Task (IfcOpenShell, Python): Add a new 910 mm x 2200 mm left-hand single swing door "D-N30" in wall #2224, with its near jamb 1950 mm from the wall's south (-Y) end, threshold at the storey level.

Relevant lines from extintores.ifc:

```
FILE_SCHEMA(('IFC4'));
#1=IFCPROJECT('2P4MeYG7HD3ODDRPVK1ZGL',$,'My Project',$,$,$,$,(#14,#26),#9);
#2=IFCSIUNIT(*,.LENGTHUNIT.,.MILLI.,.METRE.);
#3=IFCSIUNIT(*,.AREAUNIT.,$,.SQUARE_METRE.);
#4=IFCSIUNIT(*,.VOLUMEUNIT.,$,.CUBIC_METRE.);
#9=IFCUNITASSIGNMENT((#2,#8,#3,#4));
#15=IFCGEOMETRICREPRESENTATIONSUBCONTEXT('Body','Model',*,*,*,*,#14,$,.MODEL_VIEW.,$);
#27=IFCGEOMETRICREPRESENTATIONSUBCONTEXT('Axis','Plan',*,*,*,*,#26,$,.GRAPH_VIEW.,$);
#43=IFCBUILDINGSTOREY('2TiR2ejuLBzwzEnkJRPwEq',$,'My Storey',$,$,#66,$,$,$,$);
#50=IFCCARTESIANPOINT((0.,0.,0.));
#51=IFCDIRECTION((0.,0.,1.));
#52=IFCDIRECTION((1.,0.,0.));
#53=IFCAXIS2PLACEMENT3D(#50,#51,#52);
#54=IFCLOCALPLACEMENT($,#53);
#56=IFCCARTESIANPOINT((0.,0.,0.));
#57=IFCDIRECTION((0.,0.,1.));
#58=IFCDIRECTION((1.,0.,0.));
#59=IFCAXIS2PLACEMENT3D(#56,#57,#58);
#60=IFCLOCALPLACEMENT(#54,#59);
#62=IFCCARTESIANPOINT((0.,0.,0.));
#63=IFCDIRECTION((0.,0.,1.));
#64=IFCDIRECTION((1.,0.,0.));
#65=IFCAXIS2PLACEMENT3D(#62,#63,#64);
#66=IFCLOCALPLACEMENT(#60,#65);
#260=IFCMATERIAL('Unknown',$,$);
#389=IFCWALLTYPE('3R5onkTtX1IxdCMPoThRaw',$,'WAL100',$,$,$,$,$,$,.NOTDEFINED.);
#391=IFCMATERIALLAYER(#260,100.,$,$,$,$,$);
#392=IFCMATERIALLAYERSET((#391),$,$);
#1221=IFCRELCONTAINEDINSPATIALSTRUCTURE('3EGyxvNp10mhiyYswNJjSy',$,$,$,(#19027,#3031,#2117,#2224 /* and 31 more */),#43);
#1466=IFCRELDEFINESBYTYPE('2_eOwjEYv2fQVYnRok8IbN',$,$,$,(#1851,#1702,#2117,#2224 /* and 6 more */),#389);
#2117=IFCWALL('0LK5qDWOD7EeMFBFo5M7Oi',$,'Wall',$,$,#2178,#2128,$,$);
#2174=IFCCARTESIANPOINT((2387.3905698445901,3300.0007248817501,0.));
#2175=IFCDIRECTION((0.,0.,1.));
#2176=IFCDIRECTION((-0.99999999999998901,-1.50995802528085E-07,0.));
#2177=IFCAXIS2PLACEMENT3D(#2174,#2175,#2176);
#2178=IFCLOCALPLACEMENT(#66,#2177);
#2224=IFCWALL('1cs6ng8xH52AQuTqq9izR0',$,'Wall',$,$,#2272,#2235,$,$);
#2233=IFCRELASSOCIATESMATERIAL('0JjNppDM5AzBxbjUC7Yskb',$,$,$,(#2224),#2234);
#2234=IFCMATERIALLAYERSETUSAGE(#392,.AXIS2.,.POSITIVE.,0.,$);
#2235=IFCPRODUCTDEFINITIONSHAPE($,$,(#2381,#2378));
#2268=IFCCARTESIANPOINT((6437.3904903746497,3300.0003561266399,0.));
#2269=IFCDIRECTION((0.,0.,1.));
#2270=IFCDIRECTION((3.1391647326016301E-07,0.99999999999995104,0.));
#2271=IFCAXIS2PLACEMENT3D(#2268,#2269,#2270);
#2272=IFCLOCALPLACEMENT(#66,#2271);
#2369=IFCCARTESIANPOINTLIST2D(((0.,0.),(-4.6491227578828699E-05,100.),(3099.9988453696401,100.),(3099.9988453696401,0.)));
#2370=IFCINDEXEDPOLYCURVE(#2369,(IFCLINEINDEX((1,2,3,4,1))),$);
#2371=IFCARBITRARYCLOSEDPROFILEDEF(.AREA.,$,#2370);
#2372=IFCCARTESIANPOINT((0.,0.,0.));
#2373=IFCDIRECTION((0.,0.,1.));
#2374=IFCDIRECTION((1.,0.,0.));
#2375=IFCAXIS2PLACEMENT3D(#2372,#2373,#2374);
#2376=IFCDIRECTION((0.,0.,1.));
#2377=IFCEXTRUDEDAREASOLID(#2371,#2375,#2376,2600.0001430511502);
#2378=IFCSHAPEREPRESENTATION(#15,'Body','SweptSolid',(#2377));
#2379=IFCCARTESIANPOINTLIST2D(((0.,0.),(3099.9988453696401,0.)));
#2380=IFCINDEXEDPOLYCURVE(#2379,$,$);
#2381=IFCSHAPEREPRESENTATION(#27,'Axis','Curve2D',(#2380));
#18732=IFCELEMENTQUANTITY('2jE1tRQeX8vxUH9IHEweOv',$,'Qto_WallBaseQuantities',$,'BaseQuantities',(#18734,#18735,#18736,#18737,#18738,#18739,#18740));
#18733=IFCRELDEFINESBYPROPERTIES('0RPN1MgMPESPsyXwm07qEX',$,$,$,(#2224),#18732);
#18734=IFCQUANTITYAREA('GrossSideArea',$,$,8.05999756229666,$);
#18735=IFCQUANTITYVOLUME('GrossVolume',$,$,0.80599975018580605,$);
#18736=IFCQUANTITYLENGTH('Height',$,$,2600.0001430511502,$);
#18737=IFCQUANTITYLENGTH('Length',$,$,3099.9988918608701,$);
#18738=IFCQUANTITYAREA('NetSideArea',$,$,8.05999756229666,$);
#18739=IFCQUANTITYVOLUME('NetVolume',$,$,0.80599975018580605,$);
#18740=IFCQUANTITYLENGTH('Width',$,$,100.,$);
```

```python
import numpy as np
import ifcopenshell
import ifcopenshell.api.feature
import ifcopenshell.api.geometry
import ifcopenshell.api.pset
import ifcopenshell.api.root
import ifcopenshell.api.spatial
import ifcopenshell.geom
import ifcopenshell.util.element
import ifcopenshell.util.placement
import ifcopenshell.util.representation
import ifcopenshell.util.shape
import ifcopenshell.util.unit

model = ifcopenshell.open("extintores.ifc")
unit_scale = ifcopenshell.util.unit.calculate_unit_scale(model)
area_scale = ifcopenshell.util.unit.calculate_unit_scale(model, "AREAUNIT")
volume_scale = ifcopenshell.util.unit.calculate_unit_scale(model, "VOLUMEUNIT")
settings = ifcopenshell.geom.settings()


def volume(element):
    """Net volume in cubic metres, openings subtracted."""
    shape = ifcopenshell.geom.create_shape(settings, element)
    return ifcopenshell.util.shape.get_volume(shape.geometry)


wall = model.by_guid("1cs6ng8xH52AQuTqq9izR0")
storey = ifcopenshell.util.element.get_container(wall, ifc_class="IfcBuildingStorey")
context = ifcopenshell.util.representation.get_context(model, "Model", "Body", "MODEL_VIEW")
before = volume(wall)

width, height, from_end, sill = 0.91, 2.2, 1.95, 0.0  # metres

# The wall runs along its own X axis, and the end named is its -X end.
wall_shape = ifcopenshell.geom.create_shape(settings, wall)
x, y, z = ifcopenshell.util.shape.get_vertices(wall_shape.geometry).T
start = x.min() + from_end
face, thickness = float(y.min()), float(y.max() - y.min())
wall_matrix = ifcopenshell.util.placement.get_local_placement(wall.ObjectPlacement)
level = ifcopenshell.util.placement.get_local_placement(storey.ObjectPlacement)[2, 3]


def in_wall(x, y):
    """Placement at x, y metres in the wall's axes, at sill height."""
    matrix = wall_matrix.copy()
    matrix[:, 3] = wall_matrix @ np.array([x / unit_scale, y / unit_scale, 0.0, 1.0])
    matrix[2, 3] = level + sill / unit_scale
    return matrix


# Opening: a box that overshoots both wall faces by 50 mm.
opening = ifcopenshell.api.root.create_entity(model, ifc_class="IfcOpeningElement", predefined_type="OPENING")
box = ifcopenshell.api.geometry.add_wall_representation(
    model, context=context, length=width, height=height, thickness=thickness + 0.1
)
ifcopenshell.api.geometry.assign_representation(model, product=opening, representation=box)
ifcopenshell.api.geometry.edit_object_placement(model, product=opening, matrix=in_wall(start, face - 0.05), is_si=False)
ifcopenshell.api.feature.add_feature(model, feature=opening, element=wall)

door = ifcopenshell.api.root.create_entity(model, ifc_class="IfcDoor", name="D-N30", predefined_type="DOOR")
door.OverallWidth, door.OverallHeight = width / unit_scale, height / unit_scale
door.OperationType = "SINGLE_SWING_LEFT"
body = ifcopenshell.api.geometry.add_door_representation(
    model,
    context=context,
    overall_width=door.OverallWidth,
    overall_height=door.OverallHeight,
    operation_type="SINGLE_SWING_LEFT",
    lining_properties={"LiningDepth": thickness / unit_scale, "ThresholdDepth": thickness / unit_scale},
)
ifcopenshell.api.geometry.assign_representation(model, product=door, representation=body)
ifcopenshell.api.spatial.assign_container(model, products=[door], relating_structure=storey)
ifcopenshell.api.feature.add_filling(model, opening=opening, element=door)

# The lining spans the wall, so the door starts at the wall face.
ifcopenshell.api.geometry.edit_object_placement(model, product=door, matrix=in_wall(start, face), is_si=False)

after = volume(wall)

# Update the wall's stored quantities.
qto = model.by_id(ifcopenshell.util.element.get_pset(wall, "Qto_WallBaseQuantities", should_inherit=False)["id"])
ifcopenshell.api.pset.edit_qto(model, qto=qto, properties={
    "NetSideArea": after / thickness / area_scale,
    "NetVolume": after / volume_scale,
})

print(f"wall volume {before:.3f} -> {after:.3f} m3")

model.write("extintores-out.ifc")
```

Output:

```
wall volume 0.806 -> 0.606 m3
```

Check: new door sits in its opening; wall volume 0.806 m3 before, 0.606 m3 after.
